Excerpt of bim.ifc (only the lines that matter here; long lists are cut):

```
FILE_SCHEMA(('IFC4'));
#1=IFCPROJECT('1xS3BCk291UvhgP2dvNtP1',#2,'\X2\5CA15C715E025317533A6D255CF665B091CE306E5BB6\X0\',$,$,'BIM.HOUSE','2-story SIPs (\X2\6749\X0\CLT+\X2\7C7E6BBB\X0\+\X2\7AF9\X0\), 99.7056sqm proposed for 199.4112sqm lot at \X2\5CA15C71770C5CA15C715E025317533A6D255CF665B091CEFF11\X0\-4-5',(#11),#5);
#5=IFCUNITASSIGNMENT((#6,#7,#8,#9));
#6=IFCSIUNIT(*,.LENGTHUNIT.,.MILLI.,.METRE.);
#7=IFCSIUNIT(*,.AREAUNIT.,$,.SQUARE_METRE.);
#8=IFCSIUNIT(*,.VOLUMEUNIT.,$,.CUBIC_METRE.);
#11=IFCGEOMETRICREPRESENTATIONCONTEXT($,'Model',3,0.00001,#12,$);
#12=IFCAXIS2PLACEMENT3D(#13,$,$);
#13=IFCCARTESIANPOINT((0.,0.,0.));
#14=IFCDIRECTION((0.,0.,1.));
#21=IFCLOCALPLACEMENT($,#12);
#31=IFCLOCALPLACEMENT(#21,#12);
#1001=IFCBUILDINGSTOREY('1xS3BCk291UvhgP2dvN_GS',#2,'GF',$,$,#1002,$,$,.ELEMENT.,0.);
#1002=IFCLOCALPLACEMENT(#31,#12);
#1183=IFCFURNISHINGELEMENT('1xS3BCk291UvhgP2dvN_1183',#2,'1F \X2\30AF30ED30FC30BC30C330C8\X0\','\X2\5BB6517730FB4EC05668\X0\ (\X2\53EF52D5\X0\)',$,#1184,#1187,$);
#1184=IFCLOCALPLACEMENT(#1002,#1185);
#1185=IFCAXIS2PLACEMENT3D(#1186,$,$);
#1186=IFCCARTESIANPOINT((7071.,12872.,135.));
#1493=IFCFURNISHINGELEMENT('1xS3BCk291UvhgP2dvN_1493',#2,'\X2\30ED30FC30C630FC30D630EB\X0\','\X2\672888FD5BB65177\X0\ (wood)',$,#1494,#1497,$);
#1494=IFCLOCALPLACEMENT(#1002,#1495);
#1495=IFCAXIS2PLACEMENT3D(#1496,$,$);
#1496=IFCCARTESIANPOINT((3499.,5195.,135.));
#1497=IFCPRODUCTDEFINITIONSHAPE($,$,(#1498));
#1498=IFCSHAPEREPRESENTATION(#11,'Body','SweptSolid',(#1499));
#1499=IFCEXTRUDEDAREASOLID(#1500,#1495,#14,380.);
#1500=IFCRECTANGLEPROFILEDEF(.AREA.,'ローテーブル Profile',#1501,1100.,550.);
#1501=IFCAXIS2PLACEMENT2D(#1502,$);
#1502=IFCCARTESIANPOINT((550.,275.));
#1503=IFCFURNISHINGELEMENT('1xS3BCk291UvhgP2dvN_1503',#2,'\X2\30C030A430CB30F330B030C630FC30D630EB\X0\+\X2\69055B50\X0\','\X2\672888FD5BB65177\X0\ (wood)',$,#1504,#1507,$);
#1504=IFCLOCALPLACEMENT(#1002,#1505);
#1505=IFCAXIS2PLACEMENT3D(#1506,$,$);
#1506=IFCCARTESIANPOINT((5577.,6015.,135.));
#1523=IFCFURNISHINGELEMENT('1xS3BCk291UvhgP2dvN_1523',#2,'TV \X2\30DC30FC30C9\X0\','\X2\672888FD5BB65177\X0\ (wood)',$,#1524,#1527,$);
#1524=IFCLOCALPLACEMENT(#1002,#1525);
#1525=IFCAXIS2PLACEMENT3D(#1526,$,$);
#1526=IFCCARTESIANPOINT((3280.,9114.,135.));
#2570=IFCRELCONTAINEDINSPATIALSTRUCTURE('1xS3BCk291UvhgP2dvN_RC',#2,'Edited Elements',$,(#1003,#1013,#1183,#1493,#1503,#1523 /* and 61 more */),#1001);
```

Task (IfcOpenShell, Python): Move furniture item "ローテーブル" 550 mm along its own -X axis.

```python
import ifcopenshell
import ifcopenshell.api.geometry
import ifcopenshell.util.placement
import ifcopenshell.util.unit

model = ifcopenshell.open("bim.ifc")
unit_scale = ifcopenshell.util.unit.calculate_unit_scale(model)

item = model.by_guid("1xS3BCk291UvhgP2dvN_1493")
matrix = ifcopenshell.util.placement.get_local_placement(item.ObjectPlacement)
matrix[:3, 3] -= matrix[:3, 0] * 0.55 / unit_scale
ifcopenshell.api.geometry.edit_object_placement(model, product=item, matrix=matrix, is_si=False)

print(ifcopenshell.util.placement.get_local_placement(item.ObjectPlacement).round(3) + 0.0)

model.write("bim_updated.ifc")
```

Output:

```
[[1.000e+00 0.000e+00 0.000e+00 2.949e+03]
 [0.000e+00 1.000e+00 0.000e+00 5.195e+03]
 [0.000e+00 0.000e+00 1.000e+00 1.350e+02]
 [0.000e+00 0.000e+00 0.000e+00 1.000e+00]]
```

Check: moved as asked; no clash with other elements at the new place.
